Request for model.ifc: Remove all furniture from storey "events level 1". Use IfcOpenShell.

First a look at what the model holds.

```python
import ifcopenshell
import ifcopenshell.util.element

model = ifcopenshell.open("model.ifc")
print(model.schema)
storey = next(s for s in model.by_type("IfcBuildingStorey") if s.Name == "events level 1")
furniture = [e for e in ifcopenshell.util.element.get_decomposition(storey) if e.is_a("IfcFurnishingElement")]
seen = {}
for e in furniture:
    element_type = ifcopenshell.util.element.get_type(e)
    name = element_type.Name if element_type not in (None, e) else None
    seen[name] = seen.get(name, 0) + 1
for name, count in sorted(seen.items(), key=str):
    print(count, "x", name)
```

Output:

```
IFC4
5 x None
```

```python
import ifcopenshell
import ifcopenshell.api.root
import ifcopenshell.util.element

model = ifcopenshell.open("model.ifc")

storey = next(s for s in model.by_type("IfcBuildingStorey") if s.Name == "events level 1")
furniture = [e for e in ifcopenshell.util.element.get_decomposition(storey) if e.is_a("IfcFurnishingElement")]

for e in furniture:
    ifcopenshell.api.root.remove_product(model, product=e)
print(len(furniture), "removed")

model.write("model_updated.ifc")
```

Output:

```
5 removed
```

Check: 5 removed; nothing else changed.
